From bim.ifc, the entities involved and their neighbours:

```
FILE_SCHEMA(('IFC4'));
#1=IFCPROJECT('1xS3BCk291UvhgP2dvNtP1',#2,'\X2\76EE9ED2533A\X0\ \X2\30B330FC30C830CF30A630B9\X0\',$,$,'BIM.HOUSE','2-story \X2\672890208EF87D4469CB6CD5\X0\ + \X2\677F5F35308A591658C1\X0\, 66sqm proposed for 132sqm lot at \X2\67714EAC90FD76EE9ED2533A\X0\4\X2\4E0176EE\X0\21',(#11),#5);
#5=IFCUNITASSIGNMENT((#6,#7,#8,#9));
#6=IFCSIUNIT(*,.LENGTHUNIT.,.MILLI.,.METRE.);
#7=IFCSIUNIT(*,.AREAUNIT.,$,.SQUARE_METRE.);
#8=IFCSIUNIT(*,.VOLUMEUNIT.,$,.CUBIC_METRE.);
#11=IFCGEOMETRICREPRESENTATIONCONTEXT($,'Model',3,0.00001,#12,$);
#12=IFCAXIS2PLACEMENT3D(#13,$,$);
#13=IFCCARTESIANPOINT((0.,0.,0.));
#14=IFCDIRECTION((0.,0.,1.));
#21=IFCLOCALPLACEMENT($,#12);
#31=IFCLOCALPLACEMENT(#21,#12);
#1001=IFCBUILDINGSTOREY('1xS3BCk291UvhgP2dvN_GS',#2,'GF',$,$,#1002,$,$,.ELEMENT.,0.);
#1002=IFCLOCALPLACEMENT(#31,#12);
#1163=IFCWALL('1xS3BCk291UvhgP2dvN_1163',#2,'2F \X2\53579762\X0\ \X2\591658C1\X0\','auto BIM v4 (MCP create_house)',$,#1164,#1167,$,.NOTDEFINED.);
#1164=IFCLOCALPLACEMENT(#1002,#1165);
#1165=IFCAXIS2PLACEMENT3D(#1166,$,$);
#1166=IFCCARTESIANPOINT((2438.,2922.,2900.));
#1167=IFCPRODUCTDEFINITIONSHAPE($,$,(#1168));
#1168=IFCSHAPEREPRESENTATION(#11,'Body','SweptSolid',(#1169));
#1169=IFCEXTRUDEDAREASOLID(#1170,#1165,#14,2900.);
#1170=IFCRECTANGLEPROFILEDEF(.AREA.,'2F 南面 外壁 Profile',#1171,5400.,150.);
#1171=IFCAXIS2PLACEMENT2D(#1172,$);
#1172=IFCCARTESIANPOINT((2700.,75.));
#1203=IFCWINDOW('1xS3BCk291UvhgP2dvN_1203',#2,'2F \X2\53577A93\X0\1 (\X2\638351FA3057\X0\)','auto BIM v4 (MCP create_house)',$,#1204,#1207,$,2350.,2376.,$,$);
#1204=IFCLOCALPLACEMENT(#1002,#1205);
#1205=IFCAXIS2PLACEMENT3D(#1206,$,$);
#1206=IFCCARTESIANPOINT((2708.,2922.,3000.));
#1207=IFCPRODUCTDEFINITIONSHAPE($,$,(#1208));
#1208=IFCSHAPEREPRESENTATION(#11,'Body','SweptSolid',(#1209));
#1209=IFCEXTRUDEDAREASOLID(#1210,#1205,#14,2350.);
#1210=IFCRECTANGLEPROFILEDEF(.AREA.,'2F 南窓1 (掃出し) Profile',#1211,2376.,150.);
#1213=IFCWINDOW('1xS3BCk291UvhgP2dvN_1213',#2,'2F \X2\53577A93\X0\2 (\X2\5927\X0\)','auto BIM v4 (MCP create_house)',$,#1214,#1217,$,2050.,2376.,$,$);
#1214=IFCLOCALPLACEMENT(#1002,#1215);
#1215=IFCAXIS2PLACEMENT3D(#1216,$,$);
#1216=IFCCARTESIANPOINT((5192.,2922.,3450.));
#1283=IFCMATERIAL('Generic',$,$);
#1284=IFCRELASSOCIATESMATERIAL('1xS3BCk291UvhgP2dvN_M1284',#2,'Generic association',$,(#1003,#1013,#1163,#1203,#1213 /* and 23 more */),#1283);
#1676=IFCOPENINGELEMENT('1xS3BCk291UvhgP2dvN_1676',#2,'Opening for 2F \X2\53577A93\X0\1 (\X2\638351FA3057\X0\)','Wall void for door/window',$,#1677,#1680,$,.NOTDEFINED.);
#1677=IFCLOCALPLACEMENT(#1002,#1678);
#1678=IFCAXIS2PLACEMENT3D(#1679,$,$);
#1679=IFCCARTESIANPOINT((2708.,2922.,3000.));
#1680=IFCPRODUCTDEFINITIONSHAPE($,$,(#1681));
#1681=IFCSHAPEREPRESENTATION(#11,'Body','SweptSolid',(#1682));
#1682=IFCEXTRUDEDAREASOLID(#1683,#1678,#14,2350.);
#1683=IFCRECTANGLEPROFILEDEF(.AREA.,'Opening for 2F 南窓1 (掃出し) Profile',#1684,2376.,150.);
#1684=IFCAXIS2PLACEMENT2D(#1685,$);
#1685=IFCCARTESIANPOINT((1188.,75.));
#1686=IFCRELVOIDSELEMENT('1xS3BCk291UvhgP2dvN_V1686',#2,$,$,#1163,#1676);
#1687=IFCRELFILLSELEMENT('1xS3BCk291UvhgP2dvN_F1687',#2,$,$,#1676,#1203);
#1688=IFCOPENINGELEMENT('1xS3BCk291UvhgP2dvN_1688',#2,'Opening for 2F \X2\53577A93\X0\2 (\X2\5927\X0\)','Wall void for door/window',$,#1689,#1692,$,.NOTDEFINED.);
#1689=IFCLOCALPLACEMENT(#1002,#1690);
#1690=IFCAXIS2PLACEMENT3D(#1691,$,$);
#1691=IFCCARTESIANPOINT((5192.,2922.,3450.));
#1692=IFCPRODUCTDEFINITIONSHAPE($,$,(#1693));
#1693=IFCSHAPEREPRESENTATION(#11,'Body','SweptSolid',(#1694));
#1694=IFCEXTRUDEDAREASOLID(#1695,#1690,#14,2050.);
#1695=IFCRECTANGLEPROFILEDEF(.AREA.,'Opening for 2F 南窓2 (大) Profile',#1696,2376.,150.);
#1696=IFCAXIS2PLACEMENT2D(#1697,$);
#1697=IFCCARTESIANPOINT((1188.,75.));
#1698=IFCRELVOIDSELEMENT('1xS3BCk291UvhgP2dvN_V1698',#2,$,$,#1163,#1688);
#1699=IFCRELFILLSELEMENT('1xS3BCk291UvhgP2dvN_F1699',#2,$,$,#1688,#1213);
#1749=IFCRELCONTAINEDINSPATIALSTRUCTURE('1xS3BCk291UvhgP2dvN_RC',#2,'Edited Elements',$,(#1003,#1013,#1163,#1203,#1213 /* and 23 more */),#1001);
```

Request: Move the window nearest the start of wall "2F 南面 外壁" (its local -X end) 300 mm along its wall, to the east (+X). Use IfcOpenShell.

```python
import ifcopenshell
import ifcopenshell.api.geometry
import ifcopenshell.util.placement
import ifcopenshell.util.unit

model = ifcopenshell.open("bim.ifc")
unit_scale = ifcopenshell.util.unit.calculate_unit_scale(model)

window = model.by_guid("1xS3BCk291UvhgP2dvN_1203")
opening = window.FillsVoids[0].RelatingOpeningElement
wall = opening.VoidsElements[0].RelatingBuildingElement

wall_matrix = ifcopenshell.util.placement.get_local_placement(wall.ObjectPlacement)
shift = wall_matrix[:3, 0] * 0.3 / unit_scale
before = ifcopenshell.util.placement.get_local_placement(window.ObjectPlacement)[:3, 3].copy()

# The window is not placed relative to its opening, so move both.
for product in (opening, window):
    matrix = ifcopenshell.util.placement.get_local_placement(product.ObjectPlacement)
    matrix[:3, 3] += shift
    ifcopenshell.api.geometry.edit_object_placement(model, product=product, matrix=matrix, is_si=False)

after = ifcopenshell.util.placement.get_local_placement(window.ObjectPlacement)[:3, 3]
print("window moved by", (after - before).round(3) + 0.0)

model.write("bim_v2.ifc")
```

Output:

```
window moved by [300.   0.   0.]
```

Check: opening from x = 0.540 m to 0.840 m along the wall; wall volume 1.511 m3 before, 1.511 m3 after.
